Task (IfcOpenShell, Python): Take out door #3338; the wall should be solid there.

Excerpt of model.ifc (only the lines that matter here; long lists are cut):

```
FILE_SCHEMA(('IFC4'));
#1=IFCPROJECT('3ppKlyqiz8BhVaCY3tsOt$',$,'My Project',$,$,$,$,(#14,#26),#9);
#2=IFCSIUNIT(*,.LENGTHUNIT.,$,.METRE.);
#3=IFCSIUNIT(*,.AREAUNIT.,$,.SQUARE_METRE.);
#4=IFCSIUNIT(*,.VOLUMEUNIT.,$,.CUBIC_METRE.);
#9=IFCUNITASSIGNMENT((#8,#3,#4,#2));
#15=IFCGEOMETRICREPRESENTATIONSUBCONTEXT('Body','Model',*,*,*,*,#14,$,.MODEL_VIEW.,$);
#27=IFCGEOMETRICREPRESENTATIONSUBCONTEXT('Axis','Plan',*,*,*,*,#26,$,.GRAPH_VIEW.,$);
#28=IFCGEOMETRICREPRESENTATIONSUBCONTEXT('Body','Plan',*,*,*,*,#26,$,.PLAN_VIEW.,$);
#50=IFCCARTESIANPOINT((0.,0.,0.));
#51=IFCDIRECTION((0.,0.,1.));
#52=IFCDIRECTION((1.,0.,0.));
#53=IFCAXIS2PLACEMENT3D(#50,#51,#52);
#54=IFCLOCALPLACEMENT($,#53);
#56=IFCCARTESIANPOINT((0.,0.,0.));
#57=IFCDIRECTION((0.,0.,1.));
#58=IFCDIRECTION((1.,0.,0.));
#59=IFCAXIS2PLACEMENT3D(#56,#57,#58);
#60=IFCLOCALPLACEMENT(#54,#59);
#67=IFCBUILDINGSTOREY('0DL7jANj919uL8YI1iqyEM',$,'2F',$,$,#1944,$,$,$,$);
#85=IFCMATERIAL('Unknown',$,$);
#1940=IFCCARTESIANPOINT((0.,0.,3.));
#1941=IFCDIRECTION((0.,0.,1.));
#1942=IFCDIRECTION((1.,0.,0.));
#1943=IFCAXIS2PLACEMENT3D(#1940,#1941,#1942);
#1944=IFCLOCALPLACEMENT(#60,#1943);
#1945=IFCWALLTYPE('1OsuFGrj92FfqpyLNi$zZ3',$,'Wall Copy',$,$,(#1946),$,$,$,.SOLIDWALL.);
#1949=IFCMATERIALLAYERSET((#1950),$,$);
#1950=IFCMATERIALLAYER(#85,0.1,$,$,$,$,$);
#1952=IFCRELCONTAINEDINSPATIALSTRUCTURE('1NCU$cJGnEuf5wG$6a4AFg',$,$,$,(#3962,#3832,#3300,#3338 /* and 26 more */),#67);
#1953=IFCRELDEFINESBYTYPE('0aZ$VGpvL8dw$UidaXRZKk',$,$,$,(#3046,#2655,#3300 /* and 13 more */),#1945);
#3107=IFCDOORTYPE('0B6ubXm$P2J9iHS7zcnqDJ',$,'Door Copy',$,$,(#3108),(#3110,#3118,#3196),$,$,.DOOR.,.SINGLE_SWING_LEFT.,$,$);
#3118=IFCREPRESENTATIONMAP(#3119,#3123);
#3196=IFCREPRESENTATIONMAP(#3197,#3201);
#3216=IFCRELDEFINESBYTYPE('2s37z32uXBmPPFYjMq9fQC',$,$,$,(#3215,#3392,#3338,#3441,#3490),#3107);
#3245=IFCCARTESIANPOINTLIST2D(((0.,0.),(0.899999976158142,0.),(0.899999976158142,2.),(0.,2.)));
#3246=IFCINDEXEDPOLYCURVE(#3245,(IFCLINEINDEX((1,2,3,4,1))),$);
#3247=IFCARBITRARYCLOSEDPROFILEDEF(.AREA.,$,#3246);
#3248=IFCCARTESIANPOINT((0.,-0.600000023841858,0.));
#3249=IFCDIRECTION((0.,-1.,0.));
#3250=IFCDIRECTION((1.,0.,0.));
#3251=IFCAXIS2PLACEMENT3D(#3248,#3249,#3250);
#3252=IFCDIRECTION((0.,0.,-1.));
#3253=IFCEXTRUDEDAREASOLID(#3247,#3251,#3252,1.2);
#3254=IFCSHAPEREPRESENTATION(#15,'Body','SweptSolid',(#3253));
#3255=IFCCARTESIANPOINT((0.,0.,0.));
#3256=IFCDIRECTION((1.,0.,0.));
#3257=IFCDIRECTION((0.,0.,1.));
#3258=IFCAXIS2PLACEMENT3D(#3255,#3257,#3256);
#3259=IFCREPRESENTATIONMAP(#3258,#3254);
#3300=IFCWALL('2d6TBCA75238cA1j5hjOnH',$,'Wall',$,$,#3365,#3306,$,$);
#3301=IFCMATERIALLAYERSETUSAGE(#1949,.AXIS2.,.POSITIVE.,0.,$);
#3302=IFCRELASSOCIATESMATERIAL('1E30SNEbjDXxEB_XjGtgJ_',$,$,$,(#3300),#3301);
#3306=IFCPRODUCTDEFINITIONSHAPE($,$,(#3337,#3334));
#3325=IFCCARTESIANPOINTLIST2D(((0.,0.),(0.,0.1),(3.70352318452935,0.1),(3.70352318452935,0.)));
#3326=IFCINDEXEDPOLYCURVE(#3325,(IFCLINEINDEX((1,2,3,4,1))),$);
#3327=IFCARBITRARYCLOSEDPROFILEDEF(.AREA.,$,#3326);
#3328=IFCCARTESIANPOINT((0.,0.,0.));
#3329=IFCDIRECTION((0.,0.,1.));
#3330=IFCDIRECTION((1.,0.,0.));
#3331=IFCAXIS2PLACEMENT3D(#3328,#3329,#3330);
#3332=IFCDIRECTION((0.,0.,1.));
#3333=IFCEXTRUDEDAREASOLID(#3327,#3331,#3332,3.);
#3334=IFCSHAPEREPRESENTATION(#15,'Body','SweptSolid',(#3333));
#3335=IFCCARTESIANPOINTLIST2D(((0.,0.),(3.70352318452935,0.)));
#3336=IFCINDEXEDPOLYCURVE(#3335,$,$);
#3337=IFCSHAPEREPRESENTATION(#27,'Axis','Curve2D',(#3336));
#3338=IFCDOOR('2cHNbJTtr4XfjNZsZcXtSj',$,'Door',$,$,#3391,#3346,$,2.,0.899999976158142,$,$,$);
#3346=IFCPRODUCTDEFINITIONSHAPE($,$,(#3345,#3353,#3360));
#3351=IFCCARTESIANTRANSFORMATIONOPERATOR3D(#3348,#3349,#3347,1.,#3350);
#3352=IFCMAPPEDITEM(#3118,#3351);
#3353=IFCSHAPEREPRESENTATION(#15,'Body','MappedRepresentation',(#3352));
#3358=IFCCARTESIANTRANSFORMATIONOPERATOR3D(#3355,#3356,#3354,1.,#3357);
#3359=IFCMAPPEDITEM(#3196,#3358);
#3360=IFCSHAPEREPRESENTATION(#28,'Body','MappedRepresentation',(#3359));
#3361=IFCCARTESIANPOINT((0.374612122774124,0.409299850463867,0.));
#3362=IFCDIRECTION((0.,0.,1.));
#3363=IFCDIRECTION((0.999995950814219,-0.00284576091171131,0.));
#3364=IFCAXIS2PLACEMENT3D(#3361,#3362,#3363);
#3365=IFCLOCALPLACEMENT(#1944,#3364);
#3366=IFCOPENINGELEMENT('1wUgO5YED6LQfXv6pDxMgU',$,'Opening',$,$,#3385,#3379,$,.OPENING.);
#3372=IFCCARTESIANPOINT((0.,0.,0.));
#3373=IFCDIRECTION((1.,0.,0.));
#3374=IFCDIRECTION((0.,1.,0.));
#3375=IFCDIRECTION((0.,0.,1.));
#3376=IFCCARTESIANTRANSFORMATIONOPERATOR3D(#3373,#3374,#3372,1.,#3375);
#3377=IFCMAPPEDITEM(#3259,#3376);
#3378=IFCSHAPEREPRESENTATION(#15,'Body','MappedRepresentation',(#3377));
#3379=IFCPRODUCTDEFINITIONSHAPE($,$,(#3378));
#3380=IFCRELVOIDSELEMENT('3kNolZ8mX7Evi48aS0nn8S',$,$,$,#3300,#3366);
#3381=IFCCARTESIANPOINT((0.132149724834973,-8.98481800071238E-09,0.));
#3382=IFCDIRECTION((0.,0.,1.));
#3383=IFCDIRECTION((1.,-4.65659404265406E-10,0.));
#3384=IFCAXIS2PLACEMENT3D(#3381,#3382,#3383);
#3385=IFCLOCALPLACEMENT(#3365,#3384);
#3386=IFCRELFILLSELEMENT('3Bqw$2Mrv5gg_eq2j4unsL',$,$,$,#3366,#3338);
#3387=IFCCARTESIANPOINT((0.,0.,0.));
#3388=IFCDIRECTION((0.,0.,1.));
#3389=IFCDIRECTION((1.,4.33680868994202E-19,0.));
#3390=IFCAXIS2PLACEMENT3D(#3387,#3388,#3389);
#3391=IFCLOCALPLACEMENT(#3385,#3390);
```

```python
import ifcopenshell
import ifcopenshell.api.feature
import ifcopenshell.api.root
import ifcopenshell.geom
import ifcopenshell.util.shape

model = ifcopenshell.open("model.ifc")
settings = ifcopenshell.geom.settings()


def volume(element):
    """Net volume in cubic metres, openings subtracted."""
    shape = ifcopenshell.geom.create_shape(settings, element)
    return ifcopenshell.util.shape.get_volume(shape.geometry)


door = model.by_guid("2cHNbJTtr4XfjNZsZcXtSj")
opening = door.FillsVoids[0].RelatingOpeningElement
wall = opening.VoidsElements[0].RelatingBuildingElement
before = volume(wall)

ifcopenshell.api.root.remove_product(model, product=door)
ifcopenshell.api.feature.remove_feature(model, feature=opening)

after = volume(wall)

print(f"wall volume {before:.3f} -> {after:.3f} m3")

model.write("model_updated.ifc")
```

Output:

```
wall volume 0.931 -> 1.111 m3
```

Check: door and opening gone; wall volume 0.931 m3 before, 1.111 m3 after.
